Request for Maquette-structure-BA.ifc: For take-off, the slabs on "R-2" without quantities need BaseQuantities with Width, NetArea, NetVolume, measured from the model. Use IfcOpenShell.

First a look at what the model holds.

```python
import ifcopenshell
import ifcopenshell.util.element
import ifcopenshell.util.unit

model = ifcopenshell.open("Maquette-structure-BA.ifc")
print(model.schema)
for unit_type in ("LENGTHUNIT", "AREAUNIT", "VOLUMEUNIT"):
    print(unit_type, ifcopenshell.util.unit.calculate_unit_scale(model, unit_type))
storey = next(s for s in model.by_type("IfcBuildingStorey") if s.Name == "R-2")
slabs = [e for e in ifcopenshell.util.element.get_decomposition(storey) if e.is_a("IfcSlab")]
for e in sorted(slabs, key=lambda e: e.id()):
    print(e.id(), e.is_a(), e.Name, list(ifcopenshell.util.element.get_psets(e, qtos_only=True)), sep=" | ")
```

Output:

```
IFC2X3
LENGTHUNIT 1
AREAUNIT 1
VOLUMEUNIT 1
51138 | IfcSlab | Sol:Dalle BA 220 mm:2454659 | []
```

```python
import ifcopenshell
import ifcopenshell.api.pset
import ifcopenshell.geom
import ifcopenshell.util.element
import ifcopenshell.util.shape
import ifcopenshell.util.unit

model = ifcopenshell.open("Maquette-structure-BA.ifc")
unit_scale = ifcopenshell.util.unit.calculate_unit_scale(model)
area_scale = ifcopenshell.util.unit.calculate_unit_scale(model, "AREAUNIT")
volume_scale = ifcopenshell.util.unit.calculate_unit_scale(model, "VOLUMEUNIT")
settings = ifcopenshell.geom.settings()

storey = next(s for s in model.by_type("IfcBuildingStorey") if s.Name == "R-2")
slabs = [e for e in ifcopenshell.util.element.get_decomposition(storey) if e.is_a("IfcSlab")]

for e in sorted(slabs, key=lambda e: e.id()):
    if ifcopenshell.util.element.get_psets(e, qtos_only=True, should_inherit=False):
        continue
    # Geometry comes back in metres, in the element's own axes.
    shape = ifcopenshell.geom.create_shape(settings, e)
    values = {
        "Width": ifcopenshell.util.shape.get_z(shape.geometry) / unit_scale,
        "NetArea": ifcopenshell.util.shape.get_footprint_area(shape.geometry) / area_scale,
        "NetVolume": ifcopenshell.util.shape.get_volume(shape.geometry) / volume_scale,
    }
    qto = ifcopenshell.api.pset.add_qto(model, product=e, name="BaseQuantities")
    ifcopenshell.api.pset.edit_qto(model, qto=qto, properties=values)
    print(e.id(), {k: round(v, 3) for k, v in values.items()})

model.write("Maquette-structure-BA_rev.ifc")
```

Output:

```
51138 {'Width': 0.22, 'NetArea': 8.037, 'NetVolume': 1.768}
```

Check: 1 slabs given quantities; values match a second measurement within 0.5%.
